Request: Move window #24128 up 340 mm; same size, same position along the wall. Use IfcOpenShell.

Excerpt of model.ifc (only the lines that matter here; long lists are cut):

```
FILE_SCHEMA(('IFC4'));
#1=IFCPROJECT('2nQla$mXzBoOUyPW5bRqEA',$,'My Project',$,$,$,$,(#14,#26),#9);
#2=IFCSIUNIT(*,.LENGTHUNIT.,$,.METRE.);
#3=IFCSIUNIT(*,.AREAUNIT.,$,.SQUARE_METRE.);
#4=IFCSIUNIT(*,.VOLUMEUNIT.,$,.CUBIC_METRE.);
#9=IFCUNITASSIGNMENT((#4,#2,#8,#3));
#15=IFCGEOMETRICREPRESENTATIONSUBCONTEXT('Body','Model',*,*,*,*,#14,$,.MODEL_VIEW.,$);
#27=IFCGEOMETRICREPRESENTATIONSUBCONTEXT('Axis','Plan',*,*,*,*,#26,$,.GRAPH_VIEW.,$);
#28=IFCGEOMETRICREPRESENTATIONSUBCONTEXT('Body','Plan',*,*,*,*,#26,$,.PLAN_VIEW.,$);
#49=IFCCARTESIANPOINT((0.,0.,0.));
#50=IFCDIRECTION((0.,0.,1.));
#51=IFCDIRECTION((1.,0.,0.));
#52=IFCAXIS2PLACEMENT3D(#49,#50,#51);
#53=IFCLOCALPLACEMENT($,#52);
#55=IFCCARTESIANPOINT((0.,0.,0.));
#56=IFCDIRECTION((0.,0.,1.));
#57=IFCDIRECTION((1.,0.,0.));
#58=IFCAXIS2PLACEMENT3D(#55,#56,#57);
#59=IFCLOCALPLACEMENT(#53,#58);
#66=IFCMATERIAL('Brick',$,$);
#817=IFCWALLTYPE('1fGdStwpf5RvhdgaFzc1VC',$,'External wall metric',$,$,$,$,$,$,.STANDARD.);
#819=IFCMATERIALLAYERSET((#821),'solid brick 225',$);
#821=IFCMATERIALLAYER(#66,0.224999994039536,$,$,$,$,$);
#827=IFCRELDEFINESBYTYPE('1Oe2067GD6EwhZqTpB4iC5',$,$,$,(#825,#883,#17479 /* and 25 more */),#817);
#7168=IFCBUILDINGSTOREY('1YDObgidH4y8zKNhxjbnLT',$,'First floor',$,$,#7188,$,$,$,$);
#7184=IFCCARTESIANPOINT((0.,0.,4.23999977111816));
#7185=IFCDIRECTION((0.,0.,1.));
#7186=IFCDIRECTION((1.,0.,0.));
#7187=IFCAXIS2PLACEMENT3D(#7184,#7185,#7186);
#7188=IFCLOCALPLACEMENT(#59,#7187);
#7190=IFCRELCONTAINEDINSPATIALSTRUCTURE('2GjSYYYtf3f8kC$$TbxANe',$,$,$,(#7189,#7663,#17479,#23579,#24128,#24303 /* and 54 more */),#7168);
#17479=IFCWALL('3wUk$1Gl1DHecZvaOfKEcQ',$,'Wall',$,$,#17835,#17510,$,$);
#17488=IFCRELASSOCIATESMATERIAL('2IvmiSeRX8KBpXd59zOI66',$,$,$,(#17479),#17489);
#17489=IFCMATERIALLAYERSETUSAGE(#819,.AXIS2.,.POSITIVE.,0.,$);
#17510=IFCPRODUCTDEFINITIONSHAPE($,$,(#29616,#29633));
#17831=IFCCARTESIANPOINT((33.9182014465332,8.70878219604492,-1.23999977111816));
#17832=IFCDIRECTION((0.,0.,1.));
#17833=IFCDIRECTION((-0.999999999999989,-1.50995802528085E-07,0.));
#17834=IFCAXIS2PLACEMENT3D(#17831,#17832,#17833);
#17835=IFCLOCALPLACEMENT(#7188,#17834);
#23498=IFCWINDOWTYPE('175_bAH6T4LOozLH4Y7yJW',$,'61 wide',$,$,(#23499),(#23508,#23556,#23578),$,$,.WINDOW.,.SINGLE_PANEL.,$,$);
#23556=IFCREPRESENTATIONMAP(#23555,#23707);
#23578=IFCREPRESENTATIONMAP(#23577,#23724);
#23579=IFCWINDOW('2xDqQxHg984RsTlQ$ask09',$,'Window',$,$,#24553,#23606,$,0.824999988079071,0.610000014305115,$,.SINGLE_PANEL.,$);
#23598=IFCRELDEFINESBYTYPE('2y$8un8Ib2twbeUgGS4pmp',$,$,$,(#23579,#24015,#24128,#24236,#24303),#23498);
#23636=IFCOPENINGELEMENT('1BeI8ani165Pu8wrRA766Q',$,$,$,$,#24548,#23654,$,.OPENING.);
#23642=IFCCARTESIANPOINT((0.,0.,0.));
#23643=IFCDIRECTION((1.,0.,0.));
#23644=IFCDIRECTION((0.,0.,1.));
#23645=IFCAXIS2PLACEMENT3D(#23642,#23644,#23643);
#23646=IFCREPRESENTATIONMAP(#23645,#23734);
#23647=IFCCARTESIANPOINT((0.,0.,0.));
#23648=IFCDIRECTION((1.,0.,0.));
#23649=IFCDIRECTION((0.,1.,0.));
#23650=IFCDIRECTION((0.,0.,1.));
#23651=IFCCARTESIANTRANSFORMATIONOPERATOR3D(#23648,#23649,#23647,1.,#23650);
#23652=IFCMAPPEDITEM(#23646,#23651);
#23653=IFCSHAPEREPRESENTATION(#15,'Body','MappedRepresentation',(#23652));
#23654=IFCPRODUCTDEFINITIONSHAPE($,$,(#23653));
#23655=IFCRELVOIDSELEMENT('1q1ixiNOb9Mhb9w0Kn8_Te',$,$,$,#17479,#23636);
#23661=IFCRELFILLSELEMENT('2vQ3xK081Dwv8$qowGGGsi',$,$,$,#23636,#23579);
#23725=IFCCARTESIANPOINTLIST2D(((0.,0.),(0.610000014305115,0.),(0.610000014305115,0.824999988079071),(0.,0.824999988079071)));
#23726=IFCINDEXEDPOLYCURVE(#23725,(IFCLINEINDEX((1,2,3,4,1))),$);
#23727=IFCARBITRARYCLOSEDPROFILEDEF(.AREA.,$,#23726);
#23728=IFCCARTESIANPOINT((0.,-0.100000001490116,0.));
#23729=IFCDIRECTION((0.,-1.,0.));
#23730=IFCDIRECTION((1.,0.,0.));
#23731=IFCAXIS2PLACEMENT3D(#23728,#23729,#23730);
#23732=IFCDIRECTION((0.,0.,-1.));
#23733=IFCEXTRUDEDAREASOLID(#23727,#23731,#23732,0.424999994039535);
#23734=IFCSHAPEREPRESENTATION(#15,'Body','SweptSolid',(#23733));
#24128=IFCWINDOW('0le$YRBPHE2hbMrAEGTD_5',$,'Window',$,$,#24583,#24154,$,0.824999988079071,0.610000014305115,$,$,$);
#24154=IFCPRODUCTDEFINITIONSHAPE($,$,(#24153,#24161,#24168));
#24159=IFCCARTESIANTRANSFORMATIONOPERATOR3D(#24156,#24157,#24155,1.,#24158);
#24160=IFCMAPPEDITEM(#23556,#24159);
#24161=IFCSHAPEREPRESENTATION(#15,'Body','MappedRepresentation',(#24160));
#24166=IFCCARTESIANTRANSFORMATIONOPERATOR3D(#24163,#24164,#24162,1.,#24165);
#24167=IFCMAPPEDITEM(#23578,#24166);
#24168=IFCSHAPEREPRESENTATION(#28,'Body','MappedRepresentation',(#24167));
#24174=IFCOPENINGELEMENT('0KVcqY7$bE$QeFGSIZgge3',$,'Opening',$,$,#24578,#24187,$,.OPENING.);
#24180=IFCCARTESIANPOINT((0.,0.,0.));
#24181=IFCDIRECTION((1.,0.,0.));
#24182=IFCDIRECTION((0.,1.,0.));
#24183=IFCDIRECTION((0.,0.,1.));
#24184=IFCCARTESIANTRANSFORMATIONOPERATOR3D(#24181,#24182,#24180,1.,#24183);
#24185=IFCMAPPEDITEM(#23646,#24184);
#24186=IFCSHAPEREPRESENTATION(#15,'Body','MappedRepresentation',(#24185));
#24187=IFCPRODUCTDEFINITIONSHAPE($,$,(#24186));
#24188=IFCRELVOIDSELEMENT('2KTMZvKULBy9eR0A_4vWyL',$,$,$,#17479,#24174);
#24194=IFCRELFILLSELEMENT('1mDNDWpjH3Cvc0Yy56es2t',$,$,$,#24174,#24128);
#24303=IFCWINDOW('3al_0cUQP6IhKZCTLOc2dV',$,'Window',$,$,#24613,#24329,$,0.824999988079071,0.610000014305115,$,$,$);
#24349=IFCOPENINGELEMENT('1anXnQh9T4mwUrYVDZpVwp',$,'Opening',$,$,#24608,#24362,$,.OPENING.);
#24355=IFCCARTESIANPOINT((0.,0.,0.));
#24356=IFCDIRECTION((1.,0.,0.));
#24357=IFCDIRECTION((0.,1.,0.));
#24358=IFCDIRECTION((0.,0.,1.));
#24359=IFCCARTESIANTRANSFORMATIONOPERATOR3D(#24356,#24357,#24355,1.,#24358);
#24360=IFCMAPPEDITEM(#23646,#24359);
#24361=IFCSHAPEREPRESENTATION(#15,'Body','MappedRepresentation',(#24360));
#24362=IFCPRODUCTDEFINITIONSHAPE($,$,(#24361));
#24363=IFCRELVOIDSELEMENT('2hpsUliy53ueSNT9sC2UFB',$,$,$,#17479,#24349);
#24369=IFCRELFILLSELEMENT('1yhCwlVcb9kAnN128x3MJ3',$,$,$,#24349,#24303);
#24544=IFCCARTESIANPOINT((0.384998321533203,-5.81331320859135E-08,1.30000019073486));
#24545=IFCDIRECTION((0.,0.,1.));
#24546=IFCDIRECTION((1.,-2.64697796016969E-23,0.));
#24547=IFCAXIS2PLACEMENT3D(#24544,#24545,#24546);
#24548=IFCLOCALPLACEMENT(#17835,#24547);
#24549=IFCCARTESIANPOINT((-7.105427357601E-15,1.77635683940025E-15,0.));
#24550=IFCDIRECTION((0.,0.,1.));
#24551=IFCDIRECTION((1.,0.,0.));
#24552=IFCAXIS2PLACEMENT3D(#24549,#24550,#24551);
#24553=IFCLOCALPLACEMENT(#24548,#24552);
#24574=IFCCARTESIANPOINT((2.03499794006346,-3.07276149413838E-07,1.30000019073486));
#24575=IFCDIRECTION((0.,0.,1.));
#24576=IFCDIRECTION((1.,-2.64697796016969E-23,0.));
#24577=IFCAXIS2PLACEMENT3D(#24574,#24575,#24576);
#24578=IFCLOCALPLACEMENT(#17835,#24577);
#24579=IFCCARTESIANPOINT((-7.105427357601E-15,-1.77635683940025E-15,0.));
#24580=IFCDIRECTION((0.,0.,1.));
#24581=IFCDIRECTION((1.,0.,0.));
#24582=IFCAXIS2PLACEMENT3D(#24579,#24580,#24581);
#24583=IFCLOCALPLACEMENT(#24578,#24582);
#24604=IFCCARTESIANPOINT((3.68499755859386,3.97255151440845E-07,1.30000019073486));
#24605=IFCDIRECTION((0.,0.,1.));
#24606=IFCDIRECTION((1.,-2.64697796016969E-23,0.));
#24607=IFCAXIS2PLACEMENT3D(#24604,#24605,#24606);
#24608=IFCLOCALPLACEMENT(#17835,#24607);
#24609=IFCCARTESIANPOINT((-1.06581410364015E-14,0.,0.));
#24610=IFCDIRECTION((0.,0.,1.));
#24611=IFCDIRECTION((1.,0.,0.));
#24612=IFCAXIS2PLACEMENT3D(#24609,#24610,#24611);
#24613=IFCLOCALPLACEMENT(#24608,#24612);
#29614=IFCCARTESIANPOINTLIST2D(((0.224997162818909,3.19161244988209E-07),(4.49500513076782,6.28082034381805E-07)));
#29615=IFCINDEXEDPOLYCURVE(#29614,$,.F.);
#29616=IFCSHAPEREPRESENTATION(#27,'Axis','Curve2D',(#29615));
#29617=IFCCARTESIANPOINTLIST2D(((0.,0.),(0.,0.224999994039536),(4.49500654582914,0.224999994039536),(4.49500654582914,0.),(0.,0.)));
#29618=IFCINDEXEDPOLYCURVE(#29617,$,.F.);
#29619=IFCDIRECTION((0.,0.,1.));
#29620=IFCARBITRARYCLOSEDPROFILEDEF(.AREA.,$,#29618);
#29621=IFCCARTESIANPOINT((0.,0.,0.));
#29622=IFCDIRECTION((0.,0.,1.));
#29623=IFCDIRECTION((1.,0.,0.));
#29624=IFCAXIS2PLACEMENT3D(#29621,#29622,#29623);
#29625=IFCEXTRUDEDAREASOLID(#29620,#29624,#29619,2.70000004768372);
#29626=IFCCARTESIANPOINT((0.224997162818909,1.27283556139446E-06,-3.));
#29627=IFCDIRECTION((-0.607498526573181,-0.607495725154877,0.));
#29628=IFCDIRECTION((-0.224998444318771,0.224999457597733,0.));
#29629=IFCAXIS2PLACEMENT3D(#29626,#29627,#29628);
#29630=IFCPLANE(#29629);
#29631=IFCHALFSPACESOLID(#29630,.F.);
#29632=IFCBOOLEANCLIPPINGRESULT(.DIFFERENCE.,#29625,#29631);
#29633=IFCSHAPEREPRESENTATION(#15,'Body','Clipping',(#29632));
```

```python
import numpy as np
import ifcopenshell
import ifcopenshell.api.geometry
import ifcopenshell.util.placement
import ifcopenshell.util.unit

model = ifcopenshell.open("model.ifc")
unit_scale = ifcopenshell.util.unit.calculate_unit_scale(model)

window = model.by_id(24128)
opening = window.FillsVoids[0].RelatingOpeningElement
dz = 0.34

shift = np.array([0.0, 0.0, dz])
# The window is placed relative to its opening, so it follows when the opening moves.
matrix = ifcopenshell.util.placement.get_local_placement(opening.ObjectPlacement)
matrix[:3, 3] += shift
ifcopenshell.api.geometry.edit_object_placement(
    model, product=opening, matrix=matrix, is_si=False, should_transform_children=True
)

print(f"moved by {dz * unit_scale:+.3f} m")

model.write("model-out.ifc")
```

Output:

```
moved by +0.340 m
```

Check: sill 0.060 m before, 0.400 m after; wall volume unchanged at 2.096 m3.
